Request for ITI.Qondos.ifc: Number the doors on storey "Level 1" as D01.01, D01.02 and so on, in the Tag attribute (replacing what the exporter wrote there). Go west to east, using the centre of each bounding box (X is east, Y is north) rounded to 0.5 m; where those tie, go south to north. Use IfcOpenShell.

First a look at what the model holds.

```python
import ifcopenshell
import ifcopenshell.util.element
import ifcopenshell.util.placement

model = ifcopenshell.open("ITI.Qondos.ifc")
print(model.schema)
storey = next(s for s in model.by_type("IfcBuildingStorey") if s.Name == "Level 1")
doors = [e for e in ifcopenshell.util.element.get_decomposition(storey) if e.is_a("IfcDoor")]
for e in sorted(doors, key=lambda e: e.id()):
    origin = ifcopenshell.util.placement.get_local_placement(e.ObjectPlacement)[:3, 3]
    print(e.id(), e.Tag, e.Name, origin.round(2) + 0.0, sep=" | ")
```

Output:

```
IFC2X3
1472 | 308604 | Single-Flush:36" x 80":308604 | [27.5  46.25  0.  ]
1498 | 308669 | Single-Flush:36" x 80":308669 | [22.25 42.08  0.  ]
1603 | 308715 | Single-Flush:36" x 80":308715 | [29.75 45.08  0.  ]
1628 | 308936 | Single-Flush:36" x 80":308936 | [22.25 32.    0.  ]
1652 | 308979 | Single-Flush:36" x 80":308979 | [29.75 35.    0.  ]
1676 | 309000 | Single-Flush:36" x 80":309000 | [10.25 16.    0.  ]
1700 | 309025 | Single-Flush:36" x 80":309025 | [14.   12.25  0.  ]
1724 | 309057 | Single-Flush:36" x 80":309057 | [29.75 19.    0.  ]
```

```python
import ifcopenshell
import ifcopenshell.geom
import ifcopenshell.util.element
import ifcopenshell.util.shape

model = ifcopenshell.open("ITI.Qondos.ifc")
settings = ifcopenshell.geom.settings()
settings.set("use-world-coords", True)


def centre(element):
    shape = ifcopenshell.geom.create_shape(settings, element)
    return ifcopenshell.util.shape.get_bbox_centroid(shape.geometry)


storey = next(s for s in model.by_type("IfcBuildingStorey") if s.Name == "Level 1")
doors = [e for e in ifcopenshell.util.element.get_decomposition(storey) if e.is_a("IfcDoor")]

# Insertion points can sit at a corner or the storey origin, so sort by the geometry (in metres).
centres = {e: centre(e) for e in doors}
doors.sort(key=lambda e: (round(centres[e][0] / 0.5), centres[e][1]))

for i, e in enumerate(doors, start=1):
    number = f"D01.{i:02d}"
    e.Tag = number
    print(e.id(), number)

model.write("ITI.Qondos_edited.ifc")
```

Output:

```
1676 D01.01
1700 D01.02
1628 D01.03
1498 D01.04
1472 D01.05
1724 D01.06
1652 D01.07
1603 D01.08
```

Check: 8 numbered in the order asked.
